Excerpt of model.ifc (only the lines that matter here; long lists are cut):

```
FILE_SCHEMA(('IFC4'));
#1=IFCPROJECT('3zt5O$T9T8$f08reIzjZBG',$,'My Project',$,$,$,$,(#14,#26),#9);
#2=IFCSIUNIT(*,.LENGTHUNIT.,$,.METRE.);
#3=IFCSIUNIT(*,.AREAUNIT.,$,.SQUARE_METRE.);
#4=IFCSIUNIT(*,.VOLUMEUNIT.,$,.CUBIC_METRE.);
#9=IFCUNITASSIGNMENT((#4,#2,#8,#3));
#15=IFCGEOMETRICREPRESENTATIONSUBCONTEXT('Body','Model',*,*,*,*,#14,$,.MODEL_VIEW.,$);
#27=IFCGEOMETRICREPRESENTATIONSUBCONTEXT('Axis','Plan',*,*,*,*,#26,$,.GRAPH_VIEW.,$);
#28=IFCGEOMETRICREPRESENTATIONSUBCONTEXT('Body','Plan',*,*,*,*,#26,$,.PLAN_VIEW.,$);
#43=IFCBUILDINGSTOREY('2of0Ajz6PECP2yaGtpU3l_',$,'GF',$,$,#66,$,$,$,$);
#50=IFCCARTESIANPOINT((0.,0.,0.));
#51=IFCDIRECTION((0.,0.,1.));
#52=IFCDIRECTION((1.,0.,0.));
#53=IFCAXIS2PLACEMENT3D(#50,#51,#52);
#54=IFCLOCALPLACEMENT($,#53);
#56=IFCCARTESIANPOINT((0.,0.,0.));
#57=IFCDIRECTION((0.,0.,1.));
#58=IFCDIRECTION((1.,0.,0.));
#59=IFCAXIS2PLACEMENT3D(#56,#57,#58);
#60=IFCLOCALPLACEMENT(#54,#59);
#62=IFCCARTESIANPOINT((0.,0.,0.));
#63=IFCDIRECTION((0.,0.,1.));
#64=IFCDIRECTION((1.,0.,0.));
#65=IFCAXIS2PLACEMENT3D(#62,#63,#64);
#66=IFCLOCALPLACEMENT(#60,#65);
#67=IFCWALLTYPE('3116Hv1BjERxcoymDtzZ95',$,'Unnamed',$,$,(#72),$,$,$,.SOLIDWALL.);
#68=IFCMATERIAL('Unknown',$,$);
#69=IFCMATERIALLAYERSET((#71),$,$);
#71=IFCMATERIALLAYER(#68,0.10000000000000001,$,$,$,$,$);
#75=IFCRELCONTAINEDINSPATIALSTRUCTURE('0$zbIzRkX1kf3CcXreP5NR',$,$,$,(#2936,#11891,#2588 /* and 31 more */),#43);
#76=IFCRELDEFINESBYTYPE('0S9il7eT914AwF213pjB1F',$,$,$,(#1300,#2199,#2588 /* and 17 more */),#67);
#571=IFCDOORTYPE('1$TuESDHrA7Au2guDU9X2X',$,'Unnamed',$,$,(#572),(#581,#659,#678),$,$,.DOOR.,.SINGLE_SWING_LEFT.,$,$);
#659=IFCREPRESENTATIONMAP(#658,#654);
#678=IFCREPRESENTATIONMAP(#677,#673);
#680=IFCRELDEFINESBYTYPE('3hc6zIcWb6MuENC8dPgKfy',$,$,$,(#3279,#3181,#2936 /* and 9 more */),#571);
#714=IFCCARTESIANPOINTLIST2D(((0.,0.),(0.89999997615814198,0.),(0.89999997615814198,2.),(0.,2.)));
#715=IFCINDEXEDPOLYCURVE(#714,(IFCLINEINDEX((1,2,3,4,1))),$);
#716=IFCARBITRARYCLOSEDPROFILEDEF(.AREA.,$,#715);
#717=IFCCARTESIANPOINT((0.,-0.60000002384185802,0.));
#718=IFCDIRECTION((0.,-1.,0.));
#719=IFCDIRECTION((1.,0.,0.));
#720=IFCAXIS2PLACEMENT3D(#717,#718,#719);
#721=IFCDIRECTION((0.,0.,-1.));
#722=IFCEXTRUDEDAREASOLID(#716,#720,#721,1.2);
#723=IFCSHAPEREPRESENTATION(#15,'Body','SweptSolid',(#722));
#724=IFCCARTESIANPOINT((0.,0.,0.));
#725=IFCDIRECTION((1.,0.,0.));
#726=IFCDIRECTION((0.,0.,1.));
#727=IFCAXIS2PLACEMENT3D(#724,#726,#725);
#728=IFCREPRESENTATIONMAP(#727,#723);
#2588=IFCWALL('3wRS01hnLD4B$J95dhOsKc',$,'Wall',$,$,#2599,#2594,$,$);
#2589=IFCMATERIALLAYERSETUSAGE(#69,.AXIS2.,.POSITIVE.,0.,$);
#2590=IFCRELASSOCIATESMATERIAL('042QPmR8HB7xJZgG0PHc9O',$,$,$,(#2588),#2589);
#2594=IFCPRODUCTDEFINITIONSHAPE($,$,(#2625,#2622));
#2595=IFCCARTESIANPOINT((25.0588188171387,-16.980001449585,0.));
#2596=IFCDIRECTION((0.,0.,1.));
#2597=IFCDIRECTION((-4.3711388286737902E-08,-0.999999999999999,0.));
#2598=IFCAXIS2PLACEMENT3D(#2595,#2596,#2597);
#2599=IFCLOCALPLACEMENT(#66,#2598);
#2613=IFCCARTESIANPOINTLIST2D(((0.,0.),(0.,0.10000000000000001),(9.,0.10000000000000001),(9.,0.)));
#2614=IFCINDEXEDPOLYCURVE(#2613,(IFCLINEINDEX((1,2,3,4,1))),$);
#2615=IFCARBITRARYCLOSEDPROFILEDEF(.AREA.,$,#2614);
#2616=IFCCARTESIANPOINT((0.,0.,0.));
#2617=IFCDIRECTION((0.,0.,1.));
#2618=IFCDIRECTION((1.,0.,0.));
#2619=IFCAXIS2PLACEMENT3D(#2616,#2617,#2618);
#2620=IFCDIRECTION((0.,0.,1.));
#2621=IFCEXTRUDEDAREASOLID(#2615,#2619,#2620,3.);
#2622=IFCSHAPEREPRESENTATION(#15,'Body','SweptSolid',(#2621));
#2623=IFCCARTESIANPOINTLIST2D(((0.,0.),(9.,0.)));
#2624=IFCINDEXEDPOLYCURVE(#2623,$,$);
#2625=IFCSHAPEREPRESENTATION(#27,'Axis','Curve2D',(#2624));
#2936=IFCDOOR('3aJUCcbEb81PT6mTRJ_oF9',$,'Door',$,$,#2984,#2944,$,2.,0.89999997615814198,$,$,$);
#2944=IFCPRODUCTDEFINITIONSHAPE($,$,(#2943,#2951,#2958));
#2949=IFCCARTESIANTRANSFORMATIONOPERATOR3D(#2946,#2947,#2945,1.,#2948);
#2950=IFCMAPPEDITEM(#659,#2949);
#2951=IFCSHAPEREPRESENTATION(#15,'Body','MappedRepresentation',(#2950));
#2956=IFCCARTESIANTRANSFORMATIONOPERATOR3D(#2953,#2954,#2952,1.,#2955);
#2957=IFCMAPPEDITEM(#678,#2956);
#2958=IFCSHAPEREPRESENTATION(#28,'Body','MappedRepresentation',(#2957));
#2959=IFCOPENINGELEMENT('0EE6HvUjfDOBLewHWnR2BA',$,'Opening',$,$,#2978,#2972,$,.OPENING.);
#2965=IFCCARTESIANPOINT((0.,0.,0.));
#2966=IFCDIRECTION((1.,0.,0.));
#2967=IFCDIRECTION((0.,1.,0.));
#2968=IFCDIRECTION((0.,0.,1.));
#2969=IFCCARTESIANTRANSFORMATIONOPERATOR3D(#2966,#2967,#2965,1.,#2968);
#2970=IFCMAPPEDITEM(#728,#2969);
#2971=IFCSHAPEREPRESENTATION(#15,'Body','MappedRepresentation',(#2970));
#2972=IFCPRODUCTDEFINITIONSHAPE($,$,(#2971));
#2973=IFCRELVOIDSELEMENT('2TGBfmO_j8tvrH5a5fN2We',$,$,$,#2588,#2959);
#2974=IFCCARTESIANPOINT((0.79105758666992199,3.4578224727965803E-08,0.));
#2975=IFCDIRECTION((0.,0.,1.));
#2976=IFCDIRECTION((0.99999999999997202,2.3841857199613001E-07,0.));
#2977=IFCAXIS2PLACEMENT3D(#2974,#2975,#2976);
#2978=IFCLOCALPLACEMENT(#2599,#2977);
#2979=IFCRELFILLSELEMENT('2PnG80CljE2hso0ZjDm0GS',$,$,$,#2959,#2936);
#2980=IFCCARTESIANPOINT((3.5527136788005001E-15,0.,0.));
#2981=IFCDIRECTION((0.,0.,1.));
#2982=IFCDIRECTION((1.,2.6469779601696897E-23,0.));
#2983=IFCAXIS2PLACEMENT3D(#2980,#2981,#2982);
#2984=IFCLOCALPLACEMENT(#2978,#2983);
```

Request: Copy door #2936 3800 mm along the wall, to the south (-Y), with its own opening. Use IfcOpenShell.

```python
import ifcopenshell
import ifcopenshell.api.feature
import ifcopenshell.api.geometry
import ifcopenshell.api.root
import ifcopenshell.geom
import ifcopenshell.util.element
import ifcopenshell.util.placement
import ifcopenshell.util.shape

model = ifcopenshell.open("model.ifc")
settings = ifcopenshell.geom.settings()


def volume(element):
    """Net volume in cubic metres, openings subtracted."""
    shape = ifcopenshell.geom.create_shape(settings, element)
    return ifcopenshell.util.shape.get_volume(shape.geometry)


door = model.by_guid("3aJUCcbEb81PT6mTRJ_oF9")
opening = door.FillsVoids[0].RelatingOpeningElement
wall = opening.VoidsElements[0].RelatingBuildingElement
before = volume(wall)
shift = ifcopenshell.util.placement.get_local_placement(wall.ObjectPlacement)[:3, 0] * 3.8

# copy_class copies the void relationship, type, container and properties, but no geometry.
new_opening = ifcopenshell.api.root.copy_class(model, product=opening)
new_opening.Representation = ifcopenshell.util.element.copy_deep(
    model, opening.Representation, exclude=["IfcGeometricRepresentationContext", "IfcRepresentationMap"]
)
new_door = ifcopenshell.api.root.copy_class(model, product=door)
new_door.Representation = ifcopenshell.util.element.copy_deep(
    model, door.Representation, exclude=["IfcGeometricRepresentationContext", "IfcRepresentationMap"]
)
ifcopenshell.api.feature.add_filling(model, opening=new_opening, element=new_door)

for old, new in ((opening, new_opening), (door, new_door)):
    matrix = ifcopenshell.util.placement.get_local_placement(old.ObjectPlacement)
    matrix[:3, 3] += shift
    ifcopenshell.api.geometry.edit_object_placement(model, product=new, matrix=matrix, is_si=False)

after = volume(wall)

print(f"wall volume {before:.3f} -> {after:.3f} m3")

model.write("model_rev.ifc")
```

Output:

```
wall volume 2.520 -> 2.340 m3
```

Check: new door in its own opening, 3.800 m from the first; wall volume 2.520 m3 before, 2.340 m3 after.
